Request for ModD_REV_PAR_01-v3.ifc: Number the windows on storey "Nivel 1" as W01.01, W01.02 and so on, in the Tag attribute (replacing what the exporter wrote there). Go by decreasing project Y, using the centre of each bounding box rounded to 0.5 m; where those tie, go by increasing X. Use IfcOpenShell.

First a look at what the model holds.

```python
import ifcopenshell
import ifcopenshell.util.element
import ifcopenshell.util.placement

model = ifcopenshell.open("ModD_REV_PAR_01-v3.ifc")
print(model.schema)
storey = next(s for s in model.by_type("IfcBuildingStorey") if s.Name == "Nivel 1")
windows = [e for e in ifcopenshell.util.element.get_decomposition(storey) if e.is_a("IfcWindow")]
for e in sorted(windows, key=lambda e: e.id()):
    origin = ifcopenshell.util.placement.get_local_placement(e.ObjectPlacement)[:3, 3]
    print(e.id(), e.Tag, e.Name, origin.round(2) + 0.0, sep=" | ")
```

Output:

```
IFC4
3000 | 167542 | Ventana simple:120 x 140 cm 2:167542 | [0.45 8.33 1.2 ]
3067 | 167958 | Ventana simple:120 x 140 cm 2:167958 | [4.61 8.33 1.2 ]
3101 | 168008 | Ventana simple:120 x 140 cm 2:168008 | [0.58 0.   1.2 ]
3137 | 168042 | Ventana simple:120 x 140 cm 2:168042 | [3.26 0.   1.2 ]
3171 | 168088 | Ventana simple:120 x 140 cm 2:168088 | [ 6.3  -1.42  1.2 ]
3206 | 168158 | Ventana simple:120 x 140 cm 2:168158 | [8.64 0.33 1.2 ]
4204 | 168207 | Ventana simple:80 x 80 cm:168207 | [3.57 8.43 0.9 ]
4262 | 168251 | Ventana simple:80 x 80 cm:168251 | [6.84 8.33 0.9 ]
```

```python
import ifcopenshell
import ifcopenshell.geom
import ifcopenshell.util.element
import ifcopenshell.util.shape

model = ifcopenshell.open("ModD_REV_PAR_01-v3.ifc")
settings = ifcopenshell.geom.settings()
settings.set("use-world-coords", True)


def centre(element):
    shape = ifcopenshell.geom.create_shape(settings, element)
    return ifcopenshell.util.shape.get_bbox_centroid(shape.geometry)


storey = next(s for s in model.by_type("IfcBuildingStorey") if s.Name == "Nivel 1")
windows = [e for e in ifcopenshell.util.element.get_decomposition(storey) if e.is_a("IfcWindow")]

# Insertion points can sit at a corner or the storey origin, so sort by the geometry (in metres).
centres = {e: centre(e) for e in windows}
windows.sort(key=lambda e: (-round(centres[e][1] / 0.5), centres[e][0]))

for i, e in enumerate(windows, start=1):
    number = f"W01.{i:02d}"
    e.Tag = number
    print(e.id(), number)

model.write("ModD_REV_PAR_01-v3_v2.ifc")
```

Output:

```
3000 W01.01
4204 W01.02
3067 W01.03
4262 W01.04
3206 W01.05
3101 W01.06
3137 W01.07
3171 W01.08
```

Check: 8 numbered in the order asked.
